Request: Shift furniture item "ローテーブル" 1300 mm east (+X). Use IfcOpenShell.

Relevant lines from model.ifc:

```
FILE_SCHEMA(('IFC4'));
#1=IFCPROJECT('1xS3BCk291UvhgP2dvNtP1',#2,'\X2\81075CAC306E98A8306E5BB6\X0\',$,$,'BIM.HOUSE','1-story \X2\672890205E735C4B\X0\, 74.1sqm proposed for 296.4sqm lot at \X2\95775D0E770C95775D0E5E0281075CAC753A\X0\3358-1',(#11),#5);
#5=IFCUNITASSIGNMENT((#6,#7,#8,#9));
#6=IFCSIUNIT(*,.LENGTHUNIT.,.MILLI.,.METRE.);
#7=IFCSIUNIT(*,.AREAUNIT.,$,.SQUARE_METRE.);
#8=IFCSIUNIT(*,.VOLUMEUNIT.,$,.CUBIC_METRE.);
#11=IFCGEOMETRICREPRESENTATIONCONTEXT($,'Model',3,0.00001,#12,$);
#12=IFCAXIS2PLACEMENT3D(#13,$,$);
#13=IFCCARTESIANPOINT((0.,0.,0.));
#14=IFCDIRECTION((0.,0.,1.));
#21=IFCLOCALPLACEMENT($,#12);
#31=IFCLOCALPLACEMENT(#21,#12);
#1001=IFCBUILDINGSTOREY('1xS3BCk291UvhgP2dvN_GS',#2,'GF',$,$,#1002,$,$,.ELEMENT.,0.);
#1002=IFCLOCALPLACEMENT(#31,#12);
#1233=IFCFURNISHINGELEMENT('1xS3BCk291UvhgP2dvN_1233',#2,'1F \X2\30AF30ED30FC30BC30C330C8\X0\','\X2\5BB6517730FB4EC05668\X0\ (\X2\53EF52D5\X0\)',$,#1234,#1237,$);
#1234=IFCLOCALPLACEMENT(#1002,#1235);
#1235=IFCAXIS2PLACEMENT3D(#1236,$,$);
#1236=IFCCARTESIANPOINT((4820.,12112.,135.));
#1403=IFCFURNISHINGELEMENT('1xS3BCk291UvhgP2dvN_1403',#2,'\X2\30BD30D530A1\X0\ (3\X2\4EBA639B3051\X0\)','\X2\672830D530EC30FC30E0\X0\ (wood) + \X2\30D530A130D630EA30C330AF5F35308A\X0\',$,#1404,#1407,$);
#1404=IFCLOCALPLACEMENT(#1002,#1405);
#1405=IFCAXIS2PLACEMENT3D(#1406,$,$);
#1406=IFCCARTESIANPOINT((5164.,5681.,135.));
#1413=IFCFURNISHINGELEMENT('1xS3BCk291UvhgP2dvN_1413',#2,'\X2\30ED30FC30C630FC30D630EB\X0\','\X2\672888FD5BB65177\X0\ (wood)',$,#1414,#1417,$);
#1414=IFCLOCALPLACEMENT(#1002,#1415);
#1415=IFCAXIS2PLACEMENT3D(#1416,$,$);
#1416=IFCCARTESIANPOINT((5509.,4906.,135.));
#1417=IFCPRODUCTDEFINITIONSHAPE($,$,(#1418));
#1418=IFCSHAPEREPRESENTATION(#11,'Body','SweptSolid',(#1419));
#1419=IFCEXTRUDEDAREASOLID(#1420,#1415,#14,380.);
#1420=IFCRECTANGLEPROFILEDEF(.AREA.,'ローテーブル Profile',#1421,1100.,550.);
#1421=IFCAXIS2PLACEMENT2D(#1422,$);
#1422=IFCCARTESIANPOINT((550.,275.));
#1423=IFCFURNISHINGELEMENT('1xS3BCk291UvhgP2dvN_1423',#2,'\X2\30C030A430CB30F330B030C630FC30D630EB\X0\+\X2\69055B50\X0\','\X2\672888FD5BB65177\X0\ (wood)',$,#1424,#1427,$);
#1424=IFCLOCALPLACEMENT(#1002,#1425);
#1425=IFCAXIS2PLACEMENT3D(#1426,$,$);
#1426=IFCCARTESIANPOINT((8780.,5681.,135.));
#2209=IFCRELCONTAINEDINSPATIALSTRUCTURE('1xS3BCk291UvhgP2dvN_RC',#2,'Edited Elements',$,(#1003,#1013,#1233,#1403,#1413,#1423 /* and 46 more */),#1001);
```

```python
import ifcopenshell
import ifcopenshell.api.geometry
import ifcopenshell.util.placement

model = ifcopenshell.open("model.ifc")

item = model.by_guid("1xS3BCk291UvhgP2dvN_1413")
matrix = ifcopenshell.util.placement.get_local_placement(item.ObjectPlacement)
matrix[0, 3] += 1300.0
ifcopenshell.api.geometry.edit_object_placement(model, product=item, matrix=matrix, is_si=False)

print(ifcopenshell.util.placement.get_local_placement(item.ObjectPlacement).round(3) + 0.0)

model.write("model_v2.ifc")
```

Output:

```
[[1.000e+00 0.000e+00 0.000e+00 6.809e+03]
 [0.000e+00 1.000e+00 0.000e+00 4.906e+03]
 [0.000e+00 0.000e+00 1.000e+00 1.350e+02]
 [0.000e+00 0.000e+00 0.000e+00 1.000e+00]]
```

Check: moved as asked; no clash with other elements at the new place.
